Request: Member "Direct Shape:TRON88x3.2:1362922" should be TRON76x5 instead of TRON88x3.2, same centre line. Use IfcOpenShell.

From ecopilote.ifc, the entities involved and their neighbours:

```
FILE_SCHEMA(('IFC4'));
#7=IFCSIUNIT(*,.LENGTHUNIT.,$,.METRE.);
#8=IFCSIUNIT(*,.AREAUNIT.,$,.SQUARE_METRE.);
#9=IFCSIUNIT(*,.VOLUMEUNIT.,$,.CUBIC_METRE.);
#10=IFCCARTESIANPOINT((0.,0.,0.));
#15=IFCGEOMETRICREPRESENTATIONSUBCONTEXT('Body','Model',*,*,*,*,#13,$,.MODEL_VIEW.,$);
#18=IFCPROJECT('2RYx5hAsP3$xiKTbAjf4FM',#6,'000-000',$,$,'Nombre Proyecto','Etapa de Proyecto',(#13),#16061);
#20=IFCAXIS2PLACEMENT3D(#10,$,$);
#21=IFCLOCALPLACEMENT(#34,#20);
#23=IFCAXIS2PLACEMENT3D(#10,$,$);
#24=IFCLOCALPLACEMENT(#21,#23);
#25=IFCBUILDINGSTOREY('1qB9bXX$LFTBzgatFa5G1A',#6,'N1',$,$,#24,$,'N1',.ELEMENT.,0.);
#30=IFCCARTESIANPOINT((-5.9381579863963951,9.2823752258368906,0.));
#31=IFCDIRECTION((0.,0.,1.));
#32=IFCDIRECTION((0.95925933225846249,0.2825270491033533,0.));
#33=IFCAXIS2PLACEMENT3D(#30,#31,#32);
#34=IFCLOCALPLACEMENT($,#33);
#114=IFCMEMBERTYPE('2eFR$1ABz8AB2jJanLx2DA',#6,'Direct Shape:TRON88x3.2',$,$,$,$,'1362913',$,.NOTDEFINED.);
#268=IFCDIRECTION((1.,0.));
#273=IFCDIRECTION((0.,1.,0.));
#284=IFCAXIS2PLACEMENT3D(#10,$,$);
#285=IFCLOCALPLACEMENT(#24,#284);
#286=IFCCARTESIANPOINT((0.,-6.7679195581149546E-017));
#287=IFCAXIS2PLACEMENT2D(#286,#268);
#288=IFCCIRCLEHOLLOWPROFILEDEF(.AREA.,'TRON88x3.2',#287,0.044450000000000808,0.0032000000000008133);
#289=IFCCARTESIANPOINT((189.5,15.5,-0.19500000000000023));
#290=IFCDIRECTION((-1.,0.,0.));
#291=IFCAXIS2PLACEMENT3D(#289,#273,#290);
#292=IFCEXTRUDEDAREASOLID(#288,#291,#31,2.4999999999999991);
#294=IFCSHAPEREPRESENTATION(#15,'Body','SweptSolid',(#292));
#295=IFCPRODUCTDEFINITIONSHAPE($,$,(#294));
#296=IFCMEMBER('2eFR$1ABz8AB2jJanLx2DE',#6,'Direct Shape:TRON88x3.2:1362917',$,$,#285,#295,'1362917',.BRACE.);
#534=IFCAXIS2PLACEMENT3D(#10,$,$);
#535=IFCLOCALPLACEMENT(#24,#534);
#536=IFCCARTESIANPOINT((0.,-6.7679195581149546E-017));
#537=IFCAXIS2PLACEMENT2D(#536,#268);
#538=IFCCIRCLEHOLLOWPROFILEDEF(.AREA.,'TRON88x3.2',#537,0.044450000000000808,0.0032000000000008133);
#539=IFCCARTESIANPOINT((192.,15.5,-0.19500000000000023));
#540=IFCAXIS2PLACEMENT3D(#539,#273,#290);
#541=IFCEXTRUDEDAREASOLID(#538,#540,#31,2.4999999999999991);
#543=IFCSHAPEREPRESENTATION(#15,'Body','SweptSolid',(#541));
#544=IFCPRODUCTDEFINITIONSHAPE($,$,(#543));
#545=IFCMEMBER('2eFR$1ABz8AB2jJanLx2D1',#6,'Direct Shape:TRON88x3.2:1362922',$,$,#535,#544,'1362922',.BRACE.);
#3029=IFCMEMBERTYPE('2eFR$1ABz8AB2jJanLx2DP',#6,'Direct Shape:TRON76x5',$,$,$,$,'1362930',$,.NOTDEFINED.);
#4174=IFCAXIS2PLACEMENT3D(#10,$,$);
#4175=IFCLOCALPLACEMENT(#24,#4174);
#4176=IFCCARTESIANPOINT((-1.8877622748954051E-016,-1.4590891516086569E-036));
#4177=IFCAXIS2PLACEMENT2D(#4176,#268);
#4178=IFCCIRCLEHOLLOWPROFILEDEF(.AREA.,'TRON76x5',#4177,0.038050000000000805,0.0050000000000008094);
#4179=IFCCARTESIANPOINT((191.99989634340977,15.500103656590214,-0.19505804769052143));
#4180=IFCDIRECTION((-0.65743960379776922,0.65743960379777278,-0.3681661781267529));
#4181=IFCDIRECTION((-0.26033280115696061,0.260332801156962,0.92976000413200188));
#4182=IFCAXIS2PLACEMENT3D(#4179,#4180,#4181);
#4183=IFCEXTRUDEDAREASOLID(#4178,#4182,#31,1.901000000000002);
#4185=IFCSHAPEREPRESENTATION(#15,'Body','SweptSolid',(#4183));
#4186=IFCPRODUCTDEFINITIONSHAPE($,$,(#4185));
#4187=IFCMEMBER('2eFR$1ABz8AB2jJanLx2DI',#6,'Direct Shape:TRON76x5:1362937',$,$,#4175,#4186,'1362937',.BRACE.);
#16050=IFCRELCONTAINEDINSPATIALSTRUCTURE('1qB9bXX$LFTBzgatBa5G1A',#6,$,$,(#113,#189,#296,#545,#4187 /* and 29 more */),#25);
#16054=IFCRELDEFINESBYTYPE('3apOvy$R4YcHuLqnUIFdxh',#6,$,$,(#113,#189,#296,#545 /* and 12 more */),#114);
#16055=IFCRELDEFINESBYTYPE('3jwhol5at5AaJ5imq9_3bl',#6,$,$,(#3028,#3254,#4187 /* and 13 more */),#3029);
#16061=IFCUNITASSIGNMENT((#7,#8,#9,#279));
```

```python
import ifcopenshell
import ifcopenshell.api.type
import ifcopenshell.util.element
import ifcopenshell.util.representation

model = ifcopenshell.open("ecopilote.ifc")

member = model.by_id(545)
source = next(p for p in model.by_type("IfcCircleHollowProfileDef") if p.ProfileName == "TRON76x5")

body = ifcopenshell.util.representation.get_representation(member, "Model", "Body")
solid = body.Items[0]
old_profile = solid.SweptArea

# Copy the section's sizes but keep this member's own profile position.
profile = ifcopenshell.util.element.copy(model, source)
profile.Position = old_profile.Position
solid.SweptArea = profile
if not model.get_total_inverses(old_profile):
    ifcopenshell.util.element.remove_deep2(model, old_profile)

new_type = model.by_guid("2eFR$1ABz8AB2jJanLx2DP")
ifcopenshell.api.type.assign_type(
    model, related_objects=[member], relating_type=new_type, should_map_representations=False
)
member.Name = member.Name.replace("TRON88x3.2", "TRON76x5")

print(solid.SweptArea)

model.write("ecopilote_updated.ifc")
```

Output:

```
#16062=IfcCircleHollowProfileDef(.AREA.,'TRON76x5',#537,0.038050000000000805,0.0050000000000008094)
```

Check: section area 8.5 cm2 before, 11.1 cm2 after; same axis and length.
